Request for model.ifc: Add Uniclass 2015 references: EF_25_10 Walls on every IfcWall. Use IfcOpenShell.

First a look at what the model holds.

```python
import ifcopenshell

model = ifcopenshell.open("model.ifc")
print(model.schema)
print("classifications:", [c.Name for c in model.by_type("IfcClassification")])
for ifc_class in ("IfcDoor", "IfcRoof", "IfcStair", "IfcWall", "IfcWindow"):
    print(ifc_class, len(model.by_type(ifc_class)))
```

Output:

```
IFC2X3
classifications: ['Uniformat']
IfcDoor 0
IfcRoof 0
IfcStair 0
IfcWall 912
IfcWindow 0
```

```python
import ifcopenshell
import ifcopenshell.api.classification

model = ifcopenshell.open("model.ifc")

# IFC2X3 requires Source and Edition and has no link from the project to the system.
system = model.create_entity("IfcClassification", Source="NBS", Edition="2015", Name="Uniclass 2015")

codes = {
    "IfcWall": ("EF_25_10", "Walls"),
}
for ifc_class, (code, name) in codes.items():
    products = model.by_type(ifc_class)
    ifcopenshell.api.classification.add_reference(
        model, products=products, classification=system, identification=code, name=name
    )
    print(code, len(products))

model.write("model_rev.ifc")
```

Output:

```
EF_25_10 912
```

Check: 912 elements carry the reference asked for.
